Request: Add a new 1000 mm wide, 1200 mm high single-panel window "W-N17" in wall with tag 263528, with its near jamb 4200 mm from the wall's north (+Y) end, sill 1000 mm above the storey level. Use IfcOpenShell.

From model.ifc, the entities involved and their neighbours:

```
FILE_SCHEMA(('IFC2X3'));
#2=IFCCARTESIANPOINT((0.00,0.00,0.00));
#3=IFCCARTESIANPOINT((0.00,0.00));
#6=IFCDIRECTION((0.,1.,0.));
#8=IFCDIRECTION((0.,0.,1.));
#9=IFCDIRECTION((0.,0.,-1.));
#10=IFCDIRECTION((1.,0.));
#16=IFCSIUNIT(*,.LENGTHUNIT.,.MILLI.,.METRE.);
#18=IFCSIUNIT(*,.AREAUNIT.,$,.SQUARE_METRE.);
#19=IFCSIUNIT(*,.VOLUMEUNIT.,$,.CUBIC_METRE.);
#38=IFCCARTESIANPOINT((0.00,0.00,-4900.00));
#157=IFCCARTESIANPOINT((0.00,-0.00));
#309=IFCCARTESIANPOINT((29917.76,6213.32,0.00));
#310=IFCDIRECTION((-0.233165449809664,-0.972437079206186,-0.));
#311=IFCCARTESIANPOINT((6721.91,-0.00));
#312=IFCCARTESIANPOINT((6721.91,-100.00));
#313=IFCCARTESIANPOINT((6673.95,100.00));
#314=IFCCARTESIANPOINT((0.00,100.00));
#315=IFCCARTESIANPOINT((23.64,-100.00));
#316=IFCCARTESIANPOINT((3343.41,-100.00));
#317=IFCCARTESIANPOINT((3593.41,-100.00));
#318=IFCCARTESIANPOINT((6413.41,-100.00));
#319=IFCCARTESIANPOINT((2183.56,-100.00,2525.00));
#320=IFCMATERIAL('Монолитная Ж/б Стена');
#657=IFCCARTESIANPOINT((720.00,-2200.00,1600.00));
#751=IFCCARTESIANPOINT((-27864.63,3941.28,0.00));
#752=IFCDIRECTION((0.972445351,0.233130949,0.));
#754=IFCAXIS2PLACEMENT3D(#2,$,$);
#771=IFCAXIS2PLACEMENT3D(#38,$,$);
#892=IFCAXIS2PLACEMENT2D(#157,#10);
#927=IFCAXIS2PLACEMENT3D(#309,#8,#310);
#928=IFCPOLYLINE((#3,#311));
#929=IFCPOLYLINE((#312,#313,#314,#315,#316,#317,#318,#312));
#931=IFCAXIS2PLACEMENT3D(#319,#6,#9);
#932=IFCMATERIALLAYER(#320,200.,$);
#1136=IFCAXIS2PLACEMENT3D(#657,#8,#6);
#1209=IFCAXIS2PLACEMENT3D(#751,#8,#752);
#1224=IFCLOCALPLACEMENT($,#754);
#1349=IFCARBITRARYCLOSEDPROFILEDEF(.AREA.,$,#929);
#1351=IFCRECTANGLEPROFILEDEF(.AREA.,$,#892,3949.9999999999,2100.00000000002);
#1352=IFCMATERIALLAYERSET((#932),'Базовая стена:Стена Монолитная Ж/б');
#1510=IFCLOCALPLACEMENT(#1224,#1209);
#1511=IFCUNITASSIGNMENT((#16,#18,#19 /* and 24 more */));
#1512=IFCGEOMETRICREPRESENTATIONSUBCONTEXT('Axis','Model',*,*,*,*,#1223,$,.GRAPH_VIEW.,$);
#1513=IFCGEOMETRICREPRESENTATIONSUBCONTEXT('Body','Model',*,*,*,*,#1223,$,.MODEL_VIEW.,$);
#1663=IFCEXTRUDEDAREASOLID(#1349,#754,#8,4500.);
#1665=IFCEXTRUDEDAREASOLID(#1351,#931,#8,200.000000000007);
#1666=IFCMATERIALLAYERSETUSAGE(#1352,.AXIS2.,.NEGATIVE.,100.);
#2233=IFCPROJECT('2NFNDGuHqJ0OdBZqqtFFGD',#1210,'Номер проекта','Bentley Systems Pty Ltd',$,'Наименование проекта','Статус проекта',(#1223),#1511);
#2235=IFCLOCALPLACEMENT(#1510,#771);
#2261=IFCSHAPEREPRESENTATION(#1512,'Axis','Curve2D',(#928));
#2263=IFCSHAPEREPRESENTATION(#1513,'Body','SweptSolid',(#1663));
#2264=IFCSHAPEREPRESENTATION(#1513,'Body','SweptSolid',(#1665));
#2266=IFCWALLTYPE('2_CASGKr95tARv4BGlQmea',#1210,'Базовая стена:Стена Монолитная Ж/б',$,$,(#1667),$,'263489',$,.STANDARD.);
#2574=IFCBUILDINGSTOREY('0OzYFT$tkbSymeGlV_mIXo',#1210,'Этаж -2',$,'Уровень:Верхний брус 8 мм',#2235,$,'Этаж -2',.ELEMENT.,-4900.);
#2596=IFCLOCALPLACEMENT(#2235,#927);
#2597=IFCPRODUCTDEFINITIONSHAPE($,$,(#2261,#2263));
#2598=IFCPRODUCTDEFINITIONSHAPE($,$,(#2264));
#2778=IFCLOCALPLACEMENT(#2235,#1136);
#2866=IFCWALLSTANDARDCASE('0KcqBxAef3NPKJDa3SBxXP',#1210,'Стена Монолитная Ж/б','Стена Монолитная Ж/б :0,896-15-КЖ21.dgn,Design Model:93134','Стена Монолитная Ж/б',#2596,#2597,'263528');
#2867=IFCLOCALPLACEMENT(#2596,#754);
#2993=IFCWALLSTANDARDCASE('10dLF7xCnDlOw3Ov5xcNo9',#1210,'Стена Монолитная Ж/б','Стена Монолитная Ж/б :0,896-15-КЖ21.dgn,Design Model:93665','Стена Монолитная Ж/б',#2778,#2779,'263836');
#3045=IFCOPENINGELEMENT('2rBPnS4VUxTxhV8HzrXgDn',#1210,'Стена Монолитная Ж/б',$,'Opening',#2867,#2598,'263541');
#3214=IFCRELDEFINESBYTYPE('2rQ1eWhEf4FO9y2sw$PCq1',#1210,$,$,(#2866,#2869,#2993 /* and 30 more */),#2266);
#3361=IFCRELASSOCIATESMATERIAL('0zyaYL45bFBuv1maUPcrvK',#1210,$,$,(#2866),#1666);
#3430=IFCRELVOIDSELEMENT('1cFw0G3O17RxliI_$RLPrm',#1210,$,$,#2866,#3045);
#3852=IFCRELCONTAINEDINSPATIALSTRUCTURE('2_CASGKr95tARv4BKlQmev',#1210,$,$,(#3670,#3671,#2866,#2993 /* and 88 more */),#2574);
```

```python
import numpy as np
import ifcopenshell
import ifcopenshell.api.feature
import ifcopenshell.api.geometry
import ifcopenshell.api.root
import ifcopenshell.api.spatial
import ifcopenshell.api.type
import ifcopenshell.geom
import ifcopenshell.util.element
import ifcopenshell.util.placement
import ifcopenshell.util.representation
import ifcopenshell.util.shape
import ifcopenshell.util.unit

model = ifcopenshell.open("model.ifc")
unit_scale = ifcopenshell.util.unit.calculate_unit_scale(model)
settings = ifcopenshell.geom.settings()


def volume(element):
    """Net volume in cubic metres, openings subtracted."""
    shape = ifcopenshell.geom.create_shape(settings, element)
    return ifcopenshell.util.shape.get_volume(shape.geometry)


wall = model.by_guid("0KcqBxAef3NPKJDa3SBxXP")
storey = ifcopenshell.util.element.get_container(wall, ifc_class="IfcBuildingStorey")
context = ifcopenshell.util.representation.get_context(model, "Model", "Body", "MODEL_VIEW")
before = volume(wall)

width, height, from_end, sill = 1, 1.2, 4.2, 1  # metres

# The wall runs along its own X axis, and the end named is its -X end.
wall_shape = ifcopenshell.geom.create_shape(settings, wall)
x, y, z = ifcopenshell.util.shape.get_vertices(wall_shape.geometry).T
start = x.min() + from_end
face, thickness = float(y.min()), float(y.max() - y.min())
wall_matrix = ifcopenshell.util.placement.get_local_placement(wall.ObjectPlacement)
level = ifcopenshell.util.placement.get_local_placement(storey.ObjectPlacement)[2, 3]


def in_wall(x, y):
    """Placement at x, y metres in the wall's axes, at sill height."""
    matrix = wall_matrix.copy()
    matrix[:, 3] = wall_matrix @ np.array([x / unit_scale, y / unit_scale, 0.0, 1.0])
    matrix[2, 3] = level + sill / unit_scale
    return matrix


# Opening: a box that overshoots both wall faces by 50 mm.
opening = ifcopenshell.api.root.create_entity(model, ifc_class="IfcOpeningElement")
box = ifcopenshell.api.geometry.add_wall_representation(
    model, context=context, length=width, height=height, thickness=thickness + 0.1
)
ifcopenshell.api.geometry.assign_representation(model, product=opening, representation=box)
ifcopenshell.api.geometry.edit_object_placement(model, product=opening, matrix=in_wall(start, face - 0.05), is_si=False)
ifcopenshell.api.feature.add_feature(model, feature=opening, element=wall)

window = ifcopenshell.api.root.create_entity(model, ifc_class="IfcWindow", name="W-N17")
window.OverallWidth, window.OverallHeight = width / unit_scale, height / unit_scale
body = ifcopenshell.api.geometry.add_window_representation(
    model,
    context=context,
    overall_width=window.OverallWidth,
    overall_height=window.OverallHeight,
    partition_type="SINGLE_PANEL",
)
ifcopenshell.api.geometry.assign_representation(model, product=window, representation=body)
ifcopenshell.api.spatial.assign_container(model, products=[window], relating_structure=storey)
fills = ifcopenshell.api.feature.add_filling(model, opening=opening, element=window)
fills.OwnerHistory = window.OwnerHistory  # required in IFC2X3

# IFC2X3 keeps the operation on the window style.
style = ifcopenshell.api.root.create_entity(model, ifc_class="IfcWindowStyle", name="W-N17")
style.OperationType, style.ConstructionType = "SINGLE_PANEL", "NOTDEFINED"
style.ParameterTakesPrecedence = style.Sizeable = False
ifcopenshell.api.type.assign_type(model, related_objects=[window], relating_type=style)

# Centre the window in the wall's thickness.
ifcopenshell.api.geometry.edit_object_placement(model, product=window, matrix=in_wall(start, face), is_si=False)
window_shape = ifcopenshell.geom.create_shape(settings, window)
depth = ifcopenshell.util.shape.get_vertices(window_shape.geometry)[:, 1]
offset = face + thickness / 2 - (depth.min() + depth.max()) / 2
ifcopenshell.api.geometry.edit_object_placement(model, product=window, matrix=in_wall(start, offset), is_si=False)

after = volume(wall)

print(f"wall volume {before:.3f} -> {after:.3f} m3")

model.write("model_edited.ifc")
```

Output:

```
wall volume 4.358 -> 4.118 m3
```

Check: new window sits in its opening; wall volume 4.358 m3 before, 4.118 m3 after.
